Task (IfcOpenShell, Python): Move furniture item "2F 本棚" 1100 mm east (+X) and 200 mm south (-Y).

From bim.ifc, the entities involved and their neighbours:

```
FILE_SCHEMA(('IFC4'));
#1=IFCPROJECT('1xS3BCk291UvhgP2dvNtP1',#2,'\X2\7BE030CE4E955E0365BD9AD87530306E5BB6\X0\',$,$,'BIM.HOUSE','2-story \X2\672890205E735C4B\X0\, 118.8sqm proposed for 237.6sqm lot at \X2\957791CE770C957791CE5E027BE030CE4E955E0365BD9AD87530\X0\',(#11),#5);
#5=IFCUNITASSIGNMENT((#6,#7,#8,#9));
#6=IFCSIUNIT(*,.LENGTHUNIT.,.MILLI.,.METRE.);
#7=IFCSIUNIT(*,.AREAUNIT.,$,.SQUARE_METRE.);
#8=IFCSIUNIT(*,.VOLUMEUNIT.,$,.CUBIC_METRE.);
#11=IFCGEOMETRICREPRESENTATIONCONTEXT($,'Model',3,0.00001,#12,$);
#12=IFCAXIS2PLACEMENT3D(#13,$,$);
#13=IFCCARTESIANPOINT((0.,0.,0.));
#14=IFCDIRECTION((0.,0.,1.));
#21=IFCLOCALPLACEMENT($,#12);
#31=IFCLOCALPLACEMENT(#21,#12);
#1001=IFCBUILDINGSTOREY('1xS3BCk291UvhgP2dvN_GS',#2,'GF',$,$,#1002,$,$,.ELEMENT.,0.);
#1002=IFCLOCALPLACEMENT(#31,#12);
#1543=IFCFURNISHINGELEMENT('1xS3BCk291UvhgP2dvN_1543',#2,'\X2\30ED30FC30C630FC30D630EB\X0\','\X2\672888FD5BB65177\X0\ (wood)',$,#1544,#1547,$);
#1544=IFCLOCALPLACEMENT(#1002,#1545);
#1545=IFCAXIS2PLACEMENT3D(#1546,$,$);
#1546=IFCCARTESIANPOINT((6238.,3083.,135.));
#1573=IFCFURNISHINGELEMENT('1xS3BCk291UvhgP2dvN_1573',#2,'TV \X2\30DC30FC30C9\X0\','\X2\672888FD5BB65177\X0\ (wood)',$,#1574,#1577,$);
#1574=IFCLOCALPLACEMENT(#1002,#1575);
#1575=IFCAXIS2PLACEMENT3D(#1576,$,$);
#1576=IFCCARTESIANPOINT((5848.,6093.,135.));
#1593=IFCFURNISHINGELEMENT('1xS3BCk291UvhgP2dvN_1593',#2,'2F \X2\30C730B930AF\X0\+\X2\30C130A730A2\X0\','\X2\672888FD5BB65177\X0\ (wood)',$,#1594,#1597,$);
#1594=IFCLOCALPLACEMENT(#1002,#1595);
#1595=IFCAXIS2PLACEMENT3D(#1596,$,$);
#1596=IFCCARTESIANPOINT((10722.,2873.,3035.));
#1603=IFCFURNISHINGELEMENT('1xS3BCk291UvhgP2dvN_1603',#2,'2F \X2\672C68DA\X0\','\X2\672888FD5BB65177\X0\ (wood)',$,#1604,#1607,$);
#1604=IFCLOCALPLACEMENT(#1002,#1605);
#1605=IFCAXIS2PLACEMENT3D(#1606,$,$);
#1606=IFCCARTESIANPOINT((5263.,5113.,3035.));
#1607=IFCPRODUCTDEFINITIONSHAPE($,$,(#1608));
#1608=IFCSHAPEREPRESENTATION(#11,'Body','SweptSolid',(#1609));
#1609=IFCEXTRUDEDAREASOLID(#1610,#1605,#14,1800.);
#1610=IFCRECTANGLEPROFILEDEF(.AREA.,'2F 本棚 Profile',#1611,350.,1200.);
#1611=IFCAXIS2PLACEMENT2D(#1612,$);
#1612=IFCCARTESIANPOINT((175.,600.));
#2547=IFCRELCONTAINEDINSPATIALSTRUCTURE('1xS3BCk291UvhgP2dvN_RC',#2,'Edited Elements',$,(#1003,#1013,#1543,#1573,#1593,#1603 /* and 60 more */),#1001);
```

```python
import ifcopenshell
import ifcopenshell.api.geometry
import ifcopenshell.util.placement
import ifcopenshell.util.unit

model = ifcopenshell.open("bim.ifc")
unit_scale = ifcopenshell.util.unit.calculate_unit_scale(model)

item = model.by_guid("1xS3BCk291UvhgP2dvN_1603")
matrix = ifcopenshell.util.placement.get_local_placement(item.ObjectPlacement)
matrix[0, 3] += 1.1 / unit_scale
matrix[1, 3] -= 0.2 / unit_scale
ifcopenshell.api.geometry.edit_object_placement(model, product=item, matrix=matrix, is_si=False)

print(ifcopenshell.util.placement.get_local_placement(item.ObjectPlacement).round(3) + 0.0)

model.write("bim_rev.ifc")
```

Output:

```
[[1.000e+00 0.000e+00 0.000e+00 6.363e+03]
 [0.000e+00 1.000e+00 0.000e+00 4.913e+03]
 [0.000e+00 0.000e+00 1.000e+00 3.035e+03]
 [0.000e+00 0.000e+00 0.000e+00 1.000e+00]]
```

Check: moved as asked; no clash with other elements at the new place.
